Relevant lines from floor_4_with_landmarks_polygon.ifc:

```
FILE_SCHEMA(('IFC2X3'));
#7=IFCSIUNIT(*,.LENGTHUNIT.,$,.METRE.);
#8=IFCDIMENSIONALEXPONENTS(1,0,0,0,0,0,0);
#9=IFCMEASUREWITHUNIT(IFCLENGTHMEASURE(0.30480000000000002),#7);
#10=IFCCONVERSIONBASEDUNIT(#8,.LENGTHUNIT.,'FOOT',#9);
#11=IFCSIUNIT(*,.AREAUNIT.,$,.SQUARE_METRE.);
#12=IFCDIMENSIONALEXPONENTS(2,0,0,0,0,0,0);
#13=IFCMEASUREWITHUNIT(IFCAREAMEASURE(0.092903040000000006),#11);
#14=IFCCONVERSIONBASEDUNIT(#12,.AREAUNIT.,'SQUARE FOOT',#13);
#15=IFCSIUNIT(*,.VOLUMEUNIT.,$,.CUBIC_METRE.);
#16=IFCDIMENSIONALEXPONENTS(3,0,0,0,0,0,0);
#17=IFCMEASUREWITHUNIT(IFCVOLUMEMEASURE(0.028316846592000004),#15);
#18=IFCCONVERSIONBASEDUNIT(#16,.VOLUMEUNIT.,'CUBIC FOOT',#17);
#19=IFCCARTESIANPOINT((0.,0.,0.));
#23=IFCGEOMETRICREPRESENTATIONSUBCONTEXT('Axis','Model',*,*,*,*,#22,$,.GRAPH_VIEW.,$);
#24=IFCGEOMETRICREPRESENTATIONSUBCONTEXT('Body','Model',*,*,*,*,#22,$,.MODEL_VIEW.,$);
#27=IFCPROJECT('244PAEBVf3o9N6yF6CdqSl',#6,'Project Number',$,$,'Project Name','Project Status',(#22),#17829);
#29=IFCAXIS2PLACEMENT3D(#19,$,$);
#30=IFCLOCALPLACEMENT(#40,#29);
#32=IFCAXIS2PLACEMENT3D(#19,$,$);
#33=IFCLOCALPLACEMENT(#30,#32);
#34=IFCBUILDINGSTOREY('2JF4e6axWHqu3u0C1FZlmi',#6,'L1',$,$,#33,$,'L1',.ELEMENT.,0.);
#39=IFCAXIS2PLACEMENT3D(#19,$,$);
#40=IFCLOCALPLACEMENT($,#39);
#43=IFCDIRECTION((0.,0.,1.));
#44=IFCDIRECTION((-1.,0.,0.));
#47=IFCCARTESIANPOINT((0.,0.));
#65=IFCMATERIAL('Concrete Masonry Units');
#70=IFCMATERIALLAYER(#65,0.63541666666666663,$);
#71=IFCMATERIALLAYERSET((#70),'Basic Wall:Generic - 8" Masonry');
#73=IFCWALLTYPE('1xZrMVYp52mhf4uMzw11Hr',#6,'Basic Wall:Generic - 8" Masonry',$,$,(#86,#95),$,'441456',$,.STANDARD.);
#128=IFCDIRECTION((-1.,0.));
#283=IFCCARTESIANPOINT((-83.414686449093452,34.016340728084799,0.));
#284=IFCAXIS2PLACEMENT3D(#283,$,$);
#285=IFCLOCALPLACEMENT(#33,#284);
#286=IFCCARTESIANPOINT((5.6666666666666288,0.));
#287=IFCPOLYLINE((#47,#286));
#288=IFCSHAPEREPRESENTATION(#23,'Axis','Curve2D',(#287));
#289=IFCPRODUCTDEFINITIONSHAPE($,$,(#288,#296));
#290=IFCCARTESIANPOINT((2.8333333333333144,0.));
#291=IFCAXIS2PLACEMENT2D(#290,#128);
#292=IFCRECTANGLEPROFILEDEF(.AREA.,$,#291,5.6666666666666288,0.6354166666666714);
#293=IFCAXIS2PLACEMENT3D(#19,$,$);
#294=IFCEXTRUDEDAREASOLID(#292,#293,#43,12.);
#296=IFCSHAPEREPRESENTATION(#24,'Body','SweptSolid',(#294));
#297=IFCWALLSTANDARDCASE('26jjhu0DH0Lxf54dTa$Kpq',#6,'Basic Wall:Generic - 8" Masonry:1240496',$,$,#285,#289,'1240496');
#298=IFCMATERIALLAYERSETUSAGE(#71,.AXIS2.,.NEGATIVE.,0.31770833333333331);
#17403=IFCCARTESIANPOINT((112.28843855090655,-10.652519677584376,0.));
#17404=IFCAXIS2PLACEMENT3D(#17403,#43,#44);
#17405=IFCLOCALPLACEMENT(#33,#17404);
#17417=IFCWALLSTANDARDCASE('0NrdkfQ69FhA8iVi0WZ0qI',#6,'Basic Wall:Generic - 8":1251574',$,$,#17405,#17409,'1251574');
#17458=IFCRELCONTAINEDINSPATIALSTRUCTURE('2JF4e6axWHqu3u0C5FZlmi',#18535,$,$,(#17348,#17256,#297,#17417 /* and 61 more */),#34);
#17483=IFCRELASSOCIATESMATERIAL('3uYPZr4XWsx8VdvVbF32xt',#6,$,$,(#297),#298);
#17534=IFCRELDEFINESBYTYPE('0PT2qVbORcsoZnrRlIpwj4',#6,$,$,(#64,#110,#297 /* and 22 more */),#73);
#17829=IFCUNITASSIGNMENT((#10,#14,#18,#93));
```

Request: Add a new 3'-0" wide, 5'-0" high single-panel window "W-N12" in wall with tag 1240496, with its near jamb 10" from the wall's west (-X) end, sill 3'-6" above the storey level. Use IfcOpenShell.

```python
import numpy as np
import ifcopenshell
import ifcopenshell.api.feature
import ifcopenshell.api.geometry
import ifcopenshell.api.root
import ifcopenshell.api.spatial
import ifcopenshell.api.type
import ifcopenshell.geom
import ifcopenshell.util.element
import ifcopenshell.util.placement
import ifcopenshell.util.representation
import ifcopenshell.util.shape
import ifcopenshell.util.unit

model = ifcopenshell.open("floor_4_with_landmarks_polygon.ifc")
unit_scale = ifcopenshell.util.unit.calculate_unit_scale(model)
settings = ifcopenshell.geom.settings()


def volume(element):
    """Net volume in cubic metres, openings subtracted."""
    shape = ifcopenshell.geom.create_shape(settings, element)
    return ifcopenshell.util.shape.get_volume(shape.geometry)


wall = model.by_guid("26jjhu0DH0Lxf54dTa$Kpq")
storey = ifcopenshell.util.element.get_container(wall, ifc_class="IfcBuildingStorey")
context = ifcopenshell.util.representation.get_context(model, "Model", "Body", "MODEL_VIEW")
before = volume(wall)

width, height, from_end, sill = 0.9144, 1.524, 0.254, 1.0668  # metres

# The wall runs along its own X axis, and the end named is its -X end.
wall_shape = ifcopenshell.geom.create_shape(settings, wall)
x, y, z = ifcopenshell.util.shape.get_vertices(wall_shape.geometry).T
start = x.min() + from_end
face, thickness = float(y.min()), float(y.max() - y.min())
wall_matrix = ifcopenshell.util.placement.get_local_placement(wall.ObjectPlacement)
level = ifcopenshell.util.placement.get_local_placement(storey.ObjectPlacement)[2, 3]


def in_wall(x, y):
    """Placement at x, y metres in the wall's axes, at sill height."""
    matrix = wall_matrix.copy()
    matrix[:, 3] = wall_matrix @ np.array([x / unit_scale, y / unit_scale, 0.0, 1.0])
    matrix[2, 3] = level + sill / unit_scale
    return matrix


# Opening: a box that overshoots both wall faces by 50 mm.
opening = ifcopenshell.api.root.create_entity(model, ifc_class="IfcOpeningElement")
box = ifcopenshell.api.geometry.add_wall_representation(
    model, context=context, length=width, height=height, thickness=thickness + 0.1
)
ifcopenshell.api.geometry.assign_representation(model, product=opening, representation=box)
ifcopenshell.api.geometry.edit_object_placement(model, product=opening, matrix=in_wall(start, face - 0.05), is_si=False)
ifcopenshell.api.feature.add_feature(model, feature=opening, element=wall)

window = ifcopenshell.api.root.create_entity(model, ifc_class="IfcWindow", name="W-N12")
window.OverallWidth, window.OverallHeight = width / unit_scale, height / unit_scale
body = ifcopenshell.api.geometry.add_window_representation(
    model,
    context=context,
    overall_width=window.OverallWidth,
    overall_height=window.OverallHeight,
    partition_type="SINGLE_PANEL",
)
ifcopenshell.api.geometry.assign_representation(model, product=window, representation=body)
ifcopenshell.api.spatial.assign_container(model, products=[window], relating_structure=storey)
fills = ifcopenshell.api.feature.add_filling(model, opening=opening, element=window)
fills.OwnerHistory = window.OwnerHistory  # required in IFC2X3

# IFC2X3 keeps the operation on the window style.
style = ifcopenshell.api.root.create_entity(model, ifc_class="IfcWindowStyle", name="W-N12")
style.OperationType, style.ConstructionType = "SINGLE_PANEL", "NOTDEFINED"
style.ParameterTakesPrecedence = style.Sizeable = False
ifcopenshell.api.type.assign_type(model, related_objects=[window], relating_type=style)

# Centre the window in the wall's thickness.
ifcopenshell.api.geometry.edit_object_placement(model, product=window, matrix=in_wall(start, face), is_si=False)
window_shape = ifcopenshell.geom.create_shape(settings, window)
depth = ifcopenshell.util.shape.get_vertices(window_shape.geometry)[:, 1]
offset = face + thickness / 2 - (depth.min() + depth.max()) / 2
ifcopenshell.api.geometry.edit_object_placement(model, product=window, matrix=in_wall(start, offset), is_si=False)

after = volume(wall)

print(f"wall volume {before:.3f} -> {after:.3f} m3")

model.write("floor_4_with_landmarks_polygon_rev.ifc")
```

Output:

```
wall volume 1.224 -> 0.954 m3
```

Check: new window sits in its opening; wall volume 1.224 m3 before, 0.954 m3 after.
